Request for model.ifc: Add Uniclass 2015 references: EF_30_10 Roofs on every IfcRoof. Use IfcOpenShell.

First a look at what the model holds.

```python
import ifcopenshell

model = ifcopenshell.open("model.ifc")
print(model.schema)
print("classifications:", [c.Name for c in model.by_type("IfcClassification")])
for ifc_class in ("IfcDoor", "IfcRoof", "IfcStair", "IfcWall", "IfcWindow"):
    print(ifc_class, len(model.by_type(ifc_class)))
```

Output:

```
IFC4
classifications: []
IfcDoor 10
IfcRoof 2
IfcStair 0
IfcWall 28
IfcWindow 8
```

```python
import ifcopenshell
import ifcopenshell.api.classification

model = ifcopenshell.open("model.ifc")

system = ifcopenshell.api.classification.add_classification(model, classification="Uniclass 2015")

codes = {
    "IfcRoof": ("EF_30_10", "Roofs"),
}
for ifc_class, (code, name) in codes.items():
    products = model.by_type(ifc_class)
    ifcopenshell.api.classification.add_reference(
        model, products=products, classification=system, identification=code, name=name
    )
    print(code, len(products))

model.write("model_updated.ifc")
```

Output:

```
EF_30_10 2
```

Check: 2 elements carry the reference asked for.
